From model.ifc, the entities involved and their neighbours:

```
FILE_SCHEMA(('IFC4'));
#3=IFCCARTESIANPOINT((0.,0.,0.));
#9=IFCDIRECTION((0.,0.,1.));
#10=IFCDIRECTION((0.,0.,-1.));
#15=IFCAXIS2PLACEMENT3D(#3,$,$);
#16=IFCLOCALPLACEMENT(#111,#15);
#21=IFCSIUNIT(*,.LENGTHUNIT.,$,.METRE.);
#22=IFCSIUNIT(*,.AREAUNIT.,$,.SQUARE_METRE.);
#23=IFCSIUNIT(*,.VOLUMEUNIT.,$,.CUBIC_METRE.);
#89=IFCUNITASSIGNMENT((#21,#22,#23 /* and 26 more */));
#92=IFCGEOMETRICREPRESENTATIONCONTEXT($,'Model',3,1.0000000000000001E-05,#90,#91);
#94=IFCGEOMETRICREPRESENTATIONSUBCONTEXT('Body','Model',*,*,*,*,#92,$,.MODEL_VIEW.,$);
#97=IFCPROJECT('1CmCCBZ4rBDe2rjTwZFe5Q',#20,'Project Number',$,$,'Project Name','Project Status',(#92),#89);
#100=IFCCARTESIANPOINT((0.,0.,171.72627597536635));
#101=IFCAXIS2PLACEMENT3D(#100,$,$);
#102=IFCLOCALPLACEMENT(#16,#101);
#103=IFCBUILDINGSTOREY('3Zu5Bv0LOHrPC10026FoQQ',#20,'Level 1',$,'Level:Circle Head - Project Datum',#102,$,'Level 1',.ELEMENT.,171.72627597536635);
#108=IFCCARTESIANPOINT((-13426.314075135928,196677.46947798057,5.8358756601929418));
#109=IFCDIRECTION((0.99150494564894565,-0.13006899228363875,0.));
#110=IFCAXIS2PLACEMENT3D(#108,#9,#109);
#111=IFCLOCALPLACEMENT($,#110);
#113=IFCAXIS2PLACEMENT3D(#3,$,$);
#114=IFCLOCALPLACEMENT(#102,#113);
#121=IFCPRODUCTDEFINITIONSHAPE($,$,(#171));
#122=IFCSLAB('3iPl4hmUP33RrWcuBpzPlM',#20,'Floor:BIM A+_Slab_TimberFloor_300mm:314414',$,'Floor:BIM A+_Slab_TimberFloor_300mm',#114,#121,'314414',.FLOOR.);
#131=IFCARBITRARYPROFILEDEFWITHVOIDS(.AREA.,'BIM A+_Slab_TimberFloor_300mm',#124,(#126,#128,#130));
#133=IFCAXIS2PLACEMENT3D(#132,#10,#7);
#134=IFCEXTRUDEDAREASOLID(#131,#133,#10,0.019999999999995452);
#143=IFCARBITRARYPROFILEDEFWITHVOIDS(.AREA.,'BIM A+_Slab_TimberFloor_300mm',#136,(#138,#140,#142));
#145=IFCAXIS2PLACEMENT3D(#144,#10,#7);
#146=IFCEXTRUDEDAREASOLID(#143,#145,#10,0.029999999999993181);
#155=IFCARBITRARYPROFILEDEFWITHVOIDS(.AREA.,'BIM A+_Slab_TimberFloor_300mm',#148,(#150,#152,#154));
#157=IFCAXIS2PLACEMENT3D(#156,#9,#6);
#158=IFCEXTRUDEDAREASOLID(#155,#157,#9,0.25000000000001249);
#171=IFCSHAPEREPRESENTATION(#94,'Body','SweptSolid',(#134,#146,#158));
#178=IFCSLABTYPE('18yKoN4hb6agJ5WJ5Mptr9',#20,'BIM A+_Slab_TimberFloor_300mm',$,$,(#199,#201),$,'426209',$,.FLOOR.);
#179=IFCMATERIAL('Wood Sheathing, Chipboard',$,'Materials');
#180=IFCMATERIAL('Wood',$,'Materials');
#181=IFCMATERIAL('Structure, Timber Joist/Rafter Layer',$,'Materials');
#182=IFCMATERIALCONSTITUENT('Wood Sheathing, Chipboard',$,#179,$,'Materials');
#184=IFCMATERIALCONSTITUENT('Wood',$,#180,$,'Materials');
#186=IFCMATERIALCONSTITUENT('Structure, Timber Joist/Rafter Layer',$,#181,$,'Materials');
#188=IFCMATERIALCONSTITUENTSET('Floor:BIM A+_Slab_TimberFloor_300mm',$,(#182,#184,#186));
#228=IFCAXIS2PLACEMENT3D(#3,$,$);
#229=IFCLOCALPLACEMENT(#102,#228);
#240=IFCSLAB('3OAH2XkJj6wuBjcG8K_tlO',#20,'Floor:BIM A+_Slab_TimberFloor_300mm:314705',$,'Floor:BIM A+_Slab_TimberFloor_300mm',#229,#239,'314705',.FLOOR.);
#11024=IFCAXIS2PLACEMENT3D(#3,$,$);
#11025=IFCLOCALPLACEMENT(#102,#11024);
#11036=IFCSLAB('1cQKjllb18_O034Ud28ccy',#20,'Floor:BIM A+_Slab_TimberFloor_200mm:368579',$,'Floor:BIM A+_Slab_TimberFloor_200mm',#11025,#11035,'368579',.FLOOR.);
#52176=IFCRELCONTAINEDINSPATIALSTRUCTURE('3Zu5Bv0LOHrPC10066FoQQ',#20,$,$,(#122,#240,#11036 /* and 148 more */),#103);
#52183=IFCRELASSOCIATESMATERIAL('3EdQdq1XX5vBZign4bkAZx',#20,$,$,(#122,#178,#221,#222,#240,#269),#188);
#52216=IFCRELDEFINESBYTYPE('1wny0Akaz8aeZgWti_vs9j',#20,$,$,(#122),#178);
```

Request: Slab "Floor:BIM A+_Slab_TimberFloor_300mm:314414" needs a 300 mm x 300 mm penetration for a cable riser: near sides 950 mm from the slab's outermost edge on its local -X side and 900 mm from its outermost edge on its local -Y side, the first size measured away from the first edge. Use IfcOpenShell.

```python
import numpy as np
import ifcopenshell
import ifcopenshell.api.feature
import ifcopenshell.api.geometry
import ifcopenshell.api.root
import ifcopenshell.geom
import ifcopenshell.util.placement
import ifcopenshell.util.representation
import ifcopenshell.util.shape
import ifcopenshell.util.unit

model = ifcopenshell.open("model.ifc")
unit_scale = ifcopenshell.util.unit.calculate_unit_scale(model)
settings = ifcopenshell.geom.settings()


def volume(element):
    """Net volume in cubic metres, openings subtracted."""
    shape = ifcopenshell.geom.create_shape(settings, element)
    return ifcopenshell.util.shape.get_volume(shape.geometry)


slab = model.by_id(122)
before = volume(slab)

# Extent in the slab's own axes, in metres. The edges named are its -X and -Y sides.
slab_shape = ifcopenshell.geom.create_shape(settings, slab)
vertices = ifcopenshell.util.shape.get_vertices(slab_shape.geometry)
x_min, y_min, bottom = vertices.min(axis=0)
top = vertices[:, 2].max()

opening = ifcopenshell.api.root.create_entity(model, ifc_class="IfcOpeningElement", name="Cable riser opening", predefined_type="OPENING")
context = ifcopenshell.util.representation.get_context(model, "Model", "Body", "MODEL_VIEW")
width, depth = 0.3, 0.3
outline = [(0.0, 0.0), (width, 0.0), (width, depth), (0.0, depth), (0.0, 0.0)]
# Overshoot both faces by 50 mm so the cut is clean.
shape = ifcopenshell.api.geometry.add_slab_representation(
    model, context=context, depth=top - bottom + 0.1, polyline=outline
)
ifcopenshell.api.geometry.assign_representation(model, product=opening, representation=shape)

matrix = ifcopenshell.util.placement.get_local_placement(slab.ObjectPlacement)
matrix[:, 3] = matrix @ np.append(np.array([x_min + 0.95, y_min + 0.9, bottom - 0.05]) / unit_scale, 1.0)
ifcopenshell.api.geometry.edit_object_placement(model, product=opening, matrix=matrix, is_si=False)
ifcopenshell.api.feature.add_feature(model, feature=opening, element=slab)

after = volume(slab)

print(f"slab volume {before:.3f} -> {after:.3f} m3")

model.write("model-out.ifc")
```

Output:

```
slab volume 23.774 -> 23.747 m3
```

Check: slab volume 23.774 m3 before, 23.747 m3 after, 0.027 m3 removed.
